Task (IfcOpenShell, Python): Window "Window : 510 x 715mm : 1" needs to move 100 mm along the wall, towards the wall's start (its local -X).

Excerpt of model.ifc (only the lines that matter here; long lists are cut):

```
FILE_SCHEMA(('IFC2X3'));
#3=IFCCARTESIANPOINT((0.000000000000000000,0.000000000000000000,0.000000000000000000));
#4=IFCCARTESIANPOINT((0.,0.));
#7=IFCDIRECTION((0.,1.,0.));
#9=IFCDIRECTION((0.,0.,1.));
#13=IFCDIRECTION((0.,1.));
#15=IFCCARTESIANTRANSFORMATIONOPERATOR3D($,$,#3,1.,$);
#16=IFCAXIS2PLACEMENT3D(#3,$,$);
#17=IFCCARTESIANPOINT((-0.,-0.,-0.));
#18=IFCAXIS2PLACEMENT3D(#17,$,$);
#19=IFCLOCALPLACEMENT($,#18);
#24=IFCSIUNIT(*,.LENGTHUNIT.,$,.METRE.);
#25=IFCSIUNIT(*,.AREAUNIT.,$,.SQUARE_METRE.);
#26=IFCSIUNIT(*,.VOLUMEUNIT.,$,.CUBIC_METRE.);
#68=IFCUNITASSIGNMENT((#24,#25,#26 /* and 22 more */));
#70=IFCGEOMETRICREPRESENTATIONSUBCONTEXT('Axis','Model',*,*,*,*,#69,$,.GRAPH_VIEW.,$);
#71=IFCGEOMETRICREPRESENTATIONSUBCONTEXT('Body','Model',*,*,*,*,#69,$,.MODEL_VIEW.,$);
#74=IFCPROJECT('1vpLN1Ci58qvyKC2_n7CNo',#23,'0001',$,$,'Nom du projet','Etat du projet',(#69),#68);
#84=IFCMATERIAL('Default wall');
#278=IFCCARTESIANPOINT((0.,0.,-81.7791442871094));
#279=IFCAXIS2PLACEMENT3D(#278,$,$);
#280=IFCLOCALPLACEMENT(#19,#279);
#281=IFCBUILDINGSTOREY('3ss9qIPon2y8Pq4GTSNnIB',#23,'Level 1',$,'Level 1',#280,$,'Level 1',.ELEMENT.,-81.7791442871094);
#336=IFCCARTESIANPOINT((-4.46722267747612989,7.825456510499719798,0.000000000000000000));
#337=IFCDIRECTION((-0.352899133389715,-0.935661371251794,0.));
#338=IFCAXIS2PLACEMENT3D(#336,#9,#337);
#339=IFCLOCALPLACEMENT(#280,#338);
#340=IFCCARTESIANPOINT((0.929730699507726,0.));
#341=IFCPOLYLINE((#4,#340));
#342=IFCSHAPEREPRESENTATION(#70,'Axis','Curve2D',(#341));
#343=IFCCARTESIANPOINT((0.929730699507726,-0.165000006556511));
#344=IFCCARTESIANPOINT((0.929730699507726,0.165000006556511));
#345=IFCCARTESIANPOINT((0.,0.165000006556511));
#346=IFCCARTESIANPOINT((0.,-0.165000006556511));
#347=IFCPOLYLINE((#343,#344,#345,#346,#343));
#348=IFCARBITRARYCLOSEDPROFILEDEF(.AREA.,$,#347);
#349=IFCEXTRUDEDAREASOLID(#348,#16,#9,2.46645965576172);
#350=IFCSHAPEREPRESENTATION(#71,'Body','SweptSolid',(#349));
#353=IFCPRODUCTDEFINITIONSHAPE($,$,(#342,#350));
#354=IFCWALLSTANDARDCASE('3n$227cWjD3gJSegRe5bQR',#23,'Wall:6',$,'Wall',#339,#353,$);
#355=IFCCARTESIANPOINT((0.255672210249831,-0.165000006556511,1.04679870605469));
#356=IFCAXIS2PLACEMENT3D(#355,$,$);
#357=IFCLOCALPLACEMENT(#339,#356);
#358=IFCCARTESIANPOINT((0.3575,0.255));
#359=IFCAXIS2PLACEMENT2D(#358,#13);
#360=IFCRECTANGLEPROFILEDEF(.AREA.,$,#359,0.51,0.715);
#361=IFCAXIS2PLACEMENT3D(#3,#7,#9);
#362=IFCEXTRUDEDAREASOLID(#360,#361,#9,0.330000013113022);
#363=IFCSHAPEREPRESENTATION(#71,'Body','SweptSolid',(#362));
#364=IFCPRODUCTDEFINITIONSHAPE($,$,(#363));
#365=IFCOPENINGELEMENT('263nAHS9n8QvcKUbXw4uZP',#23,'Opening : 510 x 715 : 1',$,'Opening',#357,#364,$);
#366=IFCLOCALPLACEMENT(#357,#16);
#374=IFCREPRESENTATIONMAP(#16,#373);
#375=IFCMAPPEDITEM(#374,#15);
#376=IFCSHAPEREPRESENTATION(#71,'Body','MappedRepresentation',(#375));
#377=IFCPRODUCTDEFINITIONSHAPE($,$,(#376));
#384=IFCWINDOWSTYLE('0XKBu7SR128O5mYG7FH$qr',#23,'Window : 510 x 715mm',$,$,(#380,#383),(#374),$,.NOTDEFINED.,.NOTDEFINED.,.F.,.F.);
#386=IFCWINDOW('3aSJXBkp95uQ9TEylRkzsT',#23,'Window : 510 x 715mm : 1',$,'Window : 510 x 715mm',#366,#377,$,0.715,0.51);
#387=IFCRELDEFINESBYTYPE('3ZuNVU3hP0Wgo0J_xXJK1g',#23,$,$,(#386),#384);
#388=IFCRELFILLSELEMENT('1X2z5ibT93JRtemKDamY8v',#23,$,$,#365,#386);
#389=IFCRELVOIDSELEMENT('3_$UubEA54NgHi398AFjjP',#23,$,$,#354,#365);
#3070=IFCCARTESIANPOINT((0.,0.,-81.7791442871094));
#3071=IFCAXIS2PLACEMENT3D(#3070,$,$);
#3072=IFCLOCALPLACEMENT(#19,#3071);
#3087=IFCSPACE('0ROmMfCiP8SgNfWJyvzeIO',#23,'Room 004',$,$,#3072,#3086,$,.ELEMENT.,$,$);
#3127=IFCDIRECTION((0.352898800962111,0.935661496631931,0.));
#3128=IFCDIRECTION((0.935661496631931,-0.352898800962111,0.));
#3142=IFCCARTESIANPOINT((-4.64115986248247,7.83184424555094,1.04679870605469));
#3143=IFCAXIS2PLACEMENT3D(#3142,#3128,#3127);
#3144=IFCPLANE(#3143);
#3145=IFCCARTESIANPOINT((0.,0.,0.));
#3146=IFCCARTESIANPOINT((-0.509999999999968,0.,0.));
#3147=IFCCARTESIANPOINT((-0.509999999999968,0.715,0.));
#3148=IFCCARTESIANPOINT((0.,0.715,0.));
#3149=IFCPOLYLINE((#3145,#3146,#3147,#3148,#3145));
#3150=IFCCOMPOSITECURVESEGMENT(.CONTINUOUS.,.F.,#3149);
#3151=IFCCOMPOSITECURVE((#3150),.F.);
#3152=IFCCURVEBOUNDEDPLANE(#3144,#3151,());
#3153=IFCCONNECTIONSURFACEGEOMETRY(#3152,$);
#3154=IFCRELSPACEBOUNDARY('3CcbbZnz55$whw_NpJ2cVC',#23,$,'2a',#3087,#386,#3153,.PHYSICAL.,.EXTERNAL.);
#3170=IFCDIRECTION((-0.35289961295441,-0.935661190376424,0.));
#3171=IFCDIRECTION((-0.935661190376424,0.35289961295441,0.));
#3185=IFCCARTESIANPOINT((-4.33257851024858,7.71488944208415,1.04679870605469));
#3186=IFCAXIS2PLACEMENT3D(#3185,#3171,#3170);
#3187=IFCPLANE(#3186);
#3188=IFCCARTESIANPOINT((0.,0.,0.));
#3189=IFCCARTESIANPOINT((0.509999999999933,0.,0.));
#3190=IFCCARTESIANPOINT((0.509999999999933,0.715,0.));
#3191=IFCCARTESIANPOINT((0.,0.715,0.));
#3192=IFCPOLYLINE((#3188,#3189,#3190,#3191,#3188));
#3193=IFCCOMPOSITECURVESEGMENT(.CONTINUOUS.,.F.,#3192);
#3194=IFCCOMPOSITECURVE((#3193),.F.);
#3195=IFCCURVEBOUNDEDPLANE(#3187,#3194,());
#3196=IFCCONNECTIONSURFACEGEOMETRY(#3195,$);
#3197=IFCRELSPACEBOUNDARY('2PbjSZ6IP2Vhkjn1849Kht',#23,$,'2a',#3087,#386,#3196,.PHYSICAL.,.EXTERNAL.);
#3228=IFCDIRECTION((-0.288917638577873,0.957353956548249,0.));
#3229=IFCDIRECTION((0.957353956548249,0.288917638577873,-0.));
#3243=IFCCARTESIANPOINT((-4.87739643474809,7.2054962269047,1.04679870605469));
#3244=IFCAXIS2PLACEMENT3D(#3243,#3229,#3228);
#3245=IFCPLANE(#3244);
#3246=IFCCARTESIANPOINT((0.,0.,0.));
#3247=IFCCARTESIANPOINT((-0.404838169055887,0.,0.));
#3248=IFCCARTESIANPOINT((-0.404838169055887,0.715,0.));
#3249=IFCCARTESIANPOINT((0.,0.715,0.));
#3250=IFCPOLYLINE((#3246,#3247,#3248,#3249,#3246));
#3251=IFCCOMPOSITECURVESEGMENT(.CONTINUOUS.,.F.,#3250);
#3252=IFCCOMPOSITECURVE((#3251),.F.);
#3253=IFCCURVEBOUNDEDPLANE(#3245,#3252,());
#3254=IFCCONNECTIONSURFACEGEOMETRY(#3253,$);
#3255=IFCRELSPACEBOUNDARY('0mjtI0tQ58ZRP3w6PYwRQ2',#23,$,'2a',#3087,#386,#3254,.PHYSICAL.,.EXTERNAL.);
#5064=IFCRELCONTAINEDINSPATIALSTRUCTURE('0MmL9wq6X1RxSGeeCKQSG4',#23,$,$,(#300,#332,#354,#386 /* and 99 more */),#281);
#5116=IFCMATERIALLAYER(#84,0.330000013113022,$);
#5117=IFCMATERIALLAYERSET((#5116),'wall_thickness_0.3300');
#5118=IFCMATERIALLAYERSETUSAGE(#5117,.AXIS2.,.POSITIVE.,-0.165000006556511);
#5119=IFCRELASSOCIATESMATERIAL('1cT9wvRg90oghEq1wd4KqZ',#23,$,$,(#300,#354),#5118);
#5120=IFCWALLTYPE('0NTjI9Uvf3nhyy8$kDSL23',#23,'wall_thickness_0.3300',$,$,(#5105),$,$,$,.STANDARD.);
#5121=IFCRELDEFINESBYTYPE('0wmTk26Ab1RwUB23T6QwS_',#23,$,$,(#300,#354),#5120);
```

```python
import numpy as np
import ifcopenshell
import ifcopenshell.api.geometry
import ifcopenshell.util.placement

model = ifcopenshell.open("model.ifc")

window = model.by_guid("3aSJXBkp95uQ9TEylRkzsT")
opening = window.FillsVoids[0].RelatingOpeningElement
wall = opening.VoidsElements[0].RelatingBuildingElement

wall_matrix = ifcopenshell.util.placement.get_local_placement(wall.ObjectPlacement)
shift = wall_matrix[:3, 0] * -0.1
before = ifcopenshell.util.placement.get_local_placement(window.ObjectPlacement)[:3, 3].copy()

# The window is placed relative to its opening, so it follows when the opening moves.
matrix = ifcopenshell.util.placement.get_local_placement(opening.ObjectPlacement)
matrix[:3, 3] += shift
ifcopenshell.api.geometry.edit_object_placement(
    model, product=opening, matrix=matrix, is_si=False, should_transform_children=True
)

# Space boundary surfaces are stored in each space's coordinates; move them too.
for rel in window.ProvidesBoundaries:
    if not rel.ConnectionGeometry:
        continue
    surface = rel.ConnectionGeometry.SurfaceOnRelatingElement.BasisSurface
    space_matrix = ifcopenshell.util.placement.get_local_placement(rel.RelatingSpace.ObjectPlacement)
    point = np.array(surface.Position.Location.Coordinates) + space_matrix[:3, :3].T @ shift
    surface.Position = model.createIfcAxis2Placement3D(
        model.createIfcCartesianPoint(point.tolist()), surface.Position.Axis, surface.Position.RefDirection
    )

after = ifcopenshell.util.placement.get_local_placement(window.ObjectPlacement)[:3, 3]
print("window moved by", (after - before).round(3) + 0.0)

model.write("model_edited.ifc")
```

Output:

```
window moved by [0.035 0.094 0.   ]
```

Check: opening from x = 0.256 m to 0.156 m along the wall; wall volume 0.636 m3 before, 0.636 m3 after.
